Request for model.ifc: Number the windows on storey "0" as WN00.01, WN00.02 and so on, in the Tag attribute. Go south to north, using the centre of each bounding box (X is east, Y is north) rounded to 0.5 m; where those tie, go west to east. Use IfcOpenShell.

First a look at what the model holds.

```python
import ifcopenshell
import ifcopenshell.util.element
import ifcopenshell.util.placement

model = ifcopenshell.open("model.ifc")
print(model.schema)
storey = next(s for s in model.by_type("IfcBuildingStorey") if s.Name == "0")
windows = [e for e in ifcopenshell.util.element.get_decomposition(storey) if e.is_a("IfcWindow")]
for e in sorted(windows, key=lambda e: e.id()):
    origin = ifcopenshell.util.placement.get_local_placement(e.ObjectPlacement)[:3, 3]
    print(e.id(), e.Tag, e.Name, origin.round(2) + 0.0, sep=" | ")
```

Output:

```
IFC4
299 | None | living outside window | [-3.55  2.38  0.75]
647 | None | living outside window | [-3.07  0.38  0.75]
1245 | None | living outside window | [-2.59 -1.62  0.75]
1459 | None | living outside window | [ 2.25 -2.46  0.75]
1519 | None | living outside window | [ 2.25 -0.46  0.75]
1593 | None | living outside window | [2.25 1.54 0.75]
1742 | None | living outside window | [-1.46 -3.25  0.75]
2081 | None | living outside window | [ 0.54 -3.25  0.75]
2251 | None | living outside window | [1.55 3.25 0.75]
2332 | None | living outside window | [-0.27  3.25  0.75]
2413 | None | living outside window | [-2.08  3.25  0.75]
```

```python
import ifcopenshell
import ifcopenshell.geom
import ifcopenshell.util.element
import ifcopenshell.util.shape

model = ifcopenshell.open("model.ifc")
settings = ifcopenshell.geom.settings()
settings.set("use-world-coords", True)


def centre(element):
    shape = ifcopenshell.geom.create_shape(settings, element)
    return ifcopenshell.util.shape.get_bbox_centroid(shape.geometry)


storey = next(s for s in model.by_type("IfcBuildingStorey") if s.Name == "0")
windows = [e for e in ifcopenshell.util.element.get_decomposition(storey) if e.is_a("IfcWindow")]

# Insertion points can sit at a corner or the storey origin, so sort by the geometry (in metres).
centres = {e: centre(e) for e in windows}
windows.sort(key=lambda e: (round(centres[e][1] / 0.5), centres[e][0]))

for i, e in enumerate(windows, start=1):
    number = f"WN00.{i:02d}"
    e.Tag = number
    print(e.id(), number)

model.write("model_updated.ifc")
```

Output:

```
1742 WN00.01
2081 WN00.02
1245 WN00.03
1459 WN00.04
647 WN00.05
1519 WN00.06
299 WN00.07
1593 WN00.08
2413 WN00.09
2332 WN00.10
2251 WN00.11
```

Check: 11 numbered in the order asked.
